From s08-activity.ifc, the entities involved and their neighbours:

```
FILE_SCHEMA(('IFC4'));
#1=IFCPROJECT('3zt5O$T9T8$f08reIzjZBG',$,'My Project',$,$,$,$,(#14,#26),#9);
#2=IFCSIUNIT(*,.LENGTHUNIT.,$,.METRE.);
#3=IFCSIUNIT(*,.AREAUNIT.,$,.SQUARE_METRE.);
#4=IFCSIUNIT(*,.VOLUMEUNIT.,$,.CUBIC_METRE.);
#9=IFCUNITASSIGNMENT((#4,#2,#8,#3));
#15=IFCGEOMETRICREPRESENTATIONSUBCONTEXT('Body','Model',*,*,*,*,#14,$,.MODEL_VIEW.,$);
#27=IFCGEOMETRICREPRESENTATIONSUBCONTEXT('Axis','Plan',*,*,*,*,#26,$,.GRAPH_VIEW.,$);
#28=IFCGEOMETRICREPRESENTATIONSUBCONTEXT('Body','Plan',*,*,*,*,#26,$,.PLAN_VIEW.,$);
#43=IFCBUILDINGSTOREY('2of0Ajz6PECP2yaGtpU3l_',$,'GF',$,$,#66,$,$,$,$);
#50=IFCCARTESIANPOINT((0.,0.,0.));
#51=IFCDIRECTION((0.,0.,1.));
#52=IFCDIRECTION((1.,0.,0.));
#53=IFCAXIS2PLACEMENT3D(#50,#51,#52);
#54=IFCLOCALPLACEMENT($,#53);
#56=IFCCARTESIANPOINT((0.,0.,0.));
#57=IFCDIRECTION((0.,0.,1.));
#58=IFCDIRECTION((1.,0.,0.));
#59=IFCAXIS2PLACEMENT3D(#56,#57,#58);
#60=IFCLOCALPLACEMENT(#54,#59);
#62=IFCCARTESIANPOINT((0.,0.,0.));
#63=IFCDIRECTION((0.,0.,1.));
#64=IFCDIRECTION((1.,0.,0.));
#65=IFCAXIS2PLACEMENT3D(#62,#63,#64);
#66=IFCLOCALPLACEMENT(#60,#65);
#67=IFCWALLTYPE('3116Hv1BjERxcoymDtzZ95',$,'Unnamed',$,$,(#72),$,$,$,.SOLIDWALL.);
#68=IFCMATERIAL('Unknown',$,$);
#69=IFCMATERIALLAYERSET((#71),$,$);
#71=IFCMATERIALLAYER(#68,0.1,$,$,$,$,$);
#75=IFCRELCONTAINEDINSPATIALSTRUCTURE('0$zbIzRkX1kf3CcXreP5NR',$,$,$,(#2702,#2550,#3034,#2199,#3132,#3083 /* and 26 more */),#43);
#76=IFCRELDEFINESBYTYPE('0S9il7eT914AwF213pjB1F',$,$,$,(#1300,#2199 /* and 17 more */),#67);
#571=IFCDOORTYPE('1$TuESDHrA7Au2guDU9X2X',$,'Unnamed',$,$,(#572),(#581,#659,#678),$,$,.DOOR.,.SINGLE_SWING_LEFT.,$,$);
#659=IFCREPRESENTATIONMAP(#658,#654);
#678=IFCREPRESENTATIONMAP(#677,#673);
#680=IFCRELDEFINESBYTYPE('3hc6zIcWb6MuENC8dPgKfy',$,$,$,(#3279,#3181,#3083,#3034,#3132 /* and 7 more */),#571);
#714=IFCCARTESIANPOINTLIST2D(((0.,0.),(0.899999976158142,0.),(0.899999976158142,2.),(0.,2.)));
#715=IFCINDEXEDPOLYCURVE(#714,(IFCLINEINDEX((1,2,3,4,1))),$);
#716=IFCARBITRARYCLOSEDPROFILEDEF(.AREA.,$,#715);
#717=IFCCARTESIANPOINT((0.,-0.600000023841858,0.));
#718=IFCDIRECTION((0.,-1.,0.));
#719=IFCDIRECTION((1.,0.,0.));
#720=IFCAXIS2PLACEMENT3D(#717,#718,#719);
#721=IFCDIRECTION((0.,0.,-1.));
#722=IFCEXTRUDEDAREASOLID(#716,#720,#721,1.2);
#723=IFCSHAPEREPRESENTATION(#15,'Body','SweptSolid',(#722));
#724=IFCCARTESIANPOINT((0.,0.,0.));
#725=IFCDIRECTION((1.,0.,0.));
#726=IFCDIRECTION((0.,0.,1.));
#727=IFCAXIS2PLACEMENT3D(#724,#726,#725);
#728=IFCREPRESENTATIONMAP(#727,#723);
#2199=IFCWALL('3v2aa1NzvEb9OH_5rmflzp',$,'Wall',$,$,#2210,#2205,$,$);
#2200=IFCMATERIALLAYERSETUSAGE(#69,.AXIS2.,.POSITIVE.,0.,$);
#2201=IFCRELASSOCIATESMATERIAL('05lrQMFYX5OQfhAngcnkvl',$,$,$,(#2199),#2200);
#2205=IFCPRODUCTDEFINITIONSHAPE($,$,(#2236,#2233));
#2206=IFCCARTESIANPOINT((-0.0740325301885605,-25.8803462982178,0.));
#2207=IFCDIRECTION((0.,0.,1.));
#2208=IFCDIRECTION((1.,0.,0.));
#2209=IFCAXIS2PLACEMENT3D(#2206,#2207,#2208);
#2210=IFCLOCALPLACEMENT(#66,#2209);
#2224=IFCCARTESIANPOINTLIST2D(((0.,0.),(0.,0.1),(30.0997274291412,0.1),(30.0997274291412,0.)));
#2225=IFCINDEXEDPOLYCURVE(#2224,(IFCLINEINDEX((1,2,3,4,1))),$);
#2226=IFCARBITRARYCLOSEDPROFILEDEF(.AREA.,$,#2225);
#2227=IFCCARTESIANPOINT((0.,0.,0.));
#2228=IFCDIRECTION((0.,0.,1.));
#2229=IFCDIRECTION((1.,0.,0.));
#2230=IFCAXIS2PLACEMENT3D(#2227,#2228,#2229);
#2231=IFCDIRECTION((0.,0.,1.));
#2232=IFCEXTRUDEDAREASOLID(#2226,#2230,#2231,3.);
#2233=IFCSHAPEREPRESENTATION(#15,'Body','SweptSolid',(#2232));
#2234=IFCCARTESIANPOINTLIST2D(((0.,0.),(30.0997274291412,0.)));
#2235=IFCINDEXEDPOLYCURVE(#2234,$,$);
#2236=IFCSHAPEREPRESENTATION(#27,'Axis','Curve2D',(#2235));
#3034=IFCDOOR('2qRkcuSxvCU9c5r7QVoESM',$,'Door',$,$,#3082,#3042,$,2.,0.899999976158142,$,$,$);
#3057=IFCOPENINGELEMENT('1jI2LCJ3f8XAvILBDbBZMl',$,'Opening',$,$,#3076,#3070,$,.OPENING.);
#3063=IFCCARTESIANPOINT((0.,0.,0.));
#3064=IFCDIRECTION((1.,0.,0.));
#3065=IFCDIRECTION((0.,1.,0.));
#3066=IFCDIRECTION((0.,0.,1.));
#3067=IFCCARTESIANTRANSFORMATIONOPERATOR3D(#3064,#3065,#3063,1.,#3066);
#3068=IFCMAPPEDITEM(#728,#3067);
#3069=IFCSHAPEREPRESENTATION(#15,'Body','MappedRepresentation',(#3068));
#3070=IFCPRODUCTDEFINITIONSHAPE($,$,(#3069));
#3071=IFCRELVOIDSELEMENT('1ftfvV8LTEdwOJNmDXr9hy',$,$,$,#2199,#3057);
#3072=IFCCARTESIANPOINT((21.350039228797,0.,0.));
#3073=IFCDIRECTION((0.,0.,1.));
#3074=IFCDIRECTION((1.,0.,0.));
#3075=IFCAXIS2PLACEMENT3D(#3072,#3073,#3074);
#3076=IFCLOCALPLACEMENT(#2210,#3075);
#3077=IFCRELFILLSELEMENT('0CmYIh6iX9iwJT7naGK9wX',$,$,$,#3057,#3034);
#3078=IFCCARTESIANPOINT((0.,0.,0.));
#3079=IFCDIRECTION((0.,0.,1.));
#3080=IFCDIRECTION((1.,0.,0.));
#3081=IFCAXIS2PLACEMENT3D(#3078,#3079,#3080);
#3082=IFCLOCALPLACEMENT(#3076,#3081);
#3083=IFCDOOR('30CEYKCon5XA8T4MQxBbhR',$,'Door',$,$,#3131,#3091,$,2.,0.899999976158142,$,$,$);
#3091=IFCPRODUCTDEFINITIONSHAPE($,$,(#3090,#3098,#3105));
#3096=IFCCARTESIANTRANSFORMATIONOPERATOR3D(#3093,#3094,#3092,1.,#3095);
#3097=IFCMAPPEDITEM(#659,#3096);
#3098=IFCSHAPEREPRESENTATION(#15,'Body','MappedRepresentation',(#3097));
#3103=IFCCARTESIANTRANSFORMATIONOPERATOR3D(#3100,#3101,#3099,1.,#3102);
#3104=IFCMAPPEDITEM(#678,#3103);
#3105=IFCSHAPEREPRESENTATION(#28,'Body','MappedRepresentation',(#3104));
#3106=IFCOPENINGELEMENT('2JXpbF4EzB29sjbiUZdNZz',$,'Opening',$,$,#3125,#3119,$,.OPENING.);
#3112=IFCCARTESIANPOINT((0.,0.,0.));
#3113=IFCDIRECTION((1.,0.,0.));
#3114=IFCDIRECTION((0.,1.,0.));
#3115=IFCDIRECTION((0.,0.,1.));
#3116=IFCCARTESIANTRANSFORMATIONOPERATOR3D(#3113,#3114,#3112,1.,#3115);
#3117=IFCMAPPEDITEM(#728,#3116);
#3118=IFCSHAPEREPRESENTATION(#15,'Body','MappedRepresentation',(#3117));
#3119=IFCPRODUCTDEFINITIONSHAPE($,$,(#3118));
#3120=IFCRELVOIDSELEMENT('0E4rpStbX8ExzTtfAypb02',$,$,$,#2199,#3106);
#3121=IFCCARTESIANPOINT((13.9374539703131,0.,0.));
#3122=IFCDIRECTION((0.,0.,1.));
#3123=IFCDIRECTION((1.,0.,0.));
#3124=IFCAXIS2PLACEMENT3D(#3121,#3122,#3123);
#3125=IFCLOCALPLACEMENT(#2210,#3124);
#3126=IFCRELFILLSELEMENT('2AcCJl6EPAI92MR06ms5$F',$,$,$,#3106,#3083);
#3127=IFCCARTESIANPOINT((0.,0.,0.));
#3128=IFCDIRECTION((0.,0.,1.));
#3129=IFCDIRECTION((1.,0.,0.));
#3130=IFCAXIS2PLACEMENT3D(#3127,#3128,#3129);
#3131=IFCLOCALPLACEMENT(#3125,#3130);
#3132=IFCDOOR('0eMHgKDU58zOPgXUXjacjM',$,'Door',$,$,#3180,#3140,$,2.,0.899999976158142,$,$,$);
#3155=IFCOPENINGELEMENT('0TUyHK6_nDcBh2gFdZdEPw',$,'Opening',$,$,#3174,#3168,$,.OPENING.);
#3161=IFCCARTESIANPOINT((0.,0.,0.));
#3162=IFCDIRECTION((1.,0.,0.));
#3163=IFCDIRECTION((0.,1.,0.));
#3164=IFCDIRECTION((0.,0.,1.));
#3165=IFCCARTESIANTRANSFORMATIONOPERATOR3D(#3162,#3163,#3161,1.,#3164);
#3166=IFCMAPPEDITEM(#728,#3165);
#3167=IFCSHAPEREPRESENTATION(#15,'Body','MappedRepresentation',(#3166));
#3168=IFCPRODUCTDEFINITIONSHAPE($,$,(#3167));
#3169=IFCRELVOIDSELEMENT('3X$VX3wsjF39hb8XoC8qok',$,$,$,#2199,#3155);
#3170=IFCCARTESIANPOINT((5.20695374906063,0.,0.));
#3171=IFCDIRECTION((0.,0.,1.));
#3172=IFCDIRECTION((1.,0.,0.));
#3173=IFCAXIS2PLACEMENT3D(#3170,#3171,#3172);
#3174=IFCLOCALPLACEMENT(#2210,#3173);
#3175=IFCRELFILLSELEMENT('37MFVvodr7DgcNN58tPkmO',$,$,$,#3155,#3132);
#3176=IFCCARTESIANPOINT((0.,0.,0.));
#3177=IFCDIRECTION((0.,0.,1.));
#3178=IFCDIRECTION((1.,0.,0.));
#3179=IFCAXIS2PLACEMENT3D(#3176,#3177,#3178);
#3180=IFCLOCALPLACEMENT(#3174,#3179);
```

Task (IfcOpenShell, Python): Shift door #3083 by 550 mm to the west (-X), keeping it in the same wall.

```python
import ifcopenshell
import ifcopenshell.api.geometry
import ifcopenshell.util.placement
import ifcopenshell.util.unit

model = ifcopenshell.open("s08-activity.ifc")
unit_scale = ifcopenshell.util.unit.calculate_unit_scale(model)

door = model.by_guid("30CEYKCon5XA8T4MQxBbhR")
opening = door.FillsVoids[0].RelatingOpeningElement
wall = opening.VoidsElements[0].RelatingBuildingElement

wall_matrix = ifcopenshell.util.placement.get_local_placement(wall.ObjectPlacement)
shift = wall_matrix[:3, 0] * -0.55 / unit_scale
before = ifcopenshell.util.placement.get_local_placement(door.ObjectPlacement)[:3, 3].copy()

# The door is placed relative to its opening, so it follows when the opening moves.
matrix = ifcopenshell.util.placement.get_local_placement(opening.ObjectPlacement)
matrix[:3, 3] += shift
ifcopenshell.api.geometry.edit_object_placement(
    model, product=opening, matrix=matrix, is_si=False, should_transform_children=True
)

after = ifcopenshell.util.placement.get_local_placement(door.ObjectPlacement)[:3, 3]
print("door moved by", (after - before).round(3) + 0.0)

model.write("s08-activity_edited.ifc")
```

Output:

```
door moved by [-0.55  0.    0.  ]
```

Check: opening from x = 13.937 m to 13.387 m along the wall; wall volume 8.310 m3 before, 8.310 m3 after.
